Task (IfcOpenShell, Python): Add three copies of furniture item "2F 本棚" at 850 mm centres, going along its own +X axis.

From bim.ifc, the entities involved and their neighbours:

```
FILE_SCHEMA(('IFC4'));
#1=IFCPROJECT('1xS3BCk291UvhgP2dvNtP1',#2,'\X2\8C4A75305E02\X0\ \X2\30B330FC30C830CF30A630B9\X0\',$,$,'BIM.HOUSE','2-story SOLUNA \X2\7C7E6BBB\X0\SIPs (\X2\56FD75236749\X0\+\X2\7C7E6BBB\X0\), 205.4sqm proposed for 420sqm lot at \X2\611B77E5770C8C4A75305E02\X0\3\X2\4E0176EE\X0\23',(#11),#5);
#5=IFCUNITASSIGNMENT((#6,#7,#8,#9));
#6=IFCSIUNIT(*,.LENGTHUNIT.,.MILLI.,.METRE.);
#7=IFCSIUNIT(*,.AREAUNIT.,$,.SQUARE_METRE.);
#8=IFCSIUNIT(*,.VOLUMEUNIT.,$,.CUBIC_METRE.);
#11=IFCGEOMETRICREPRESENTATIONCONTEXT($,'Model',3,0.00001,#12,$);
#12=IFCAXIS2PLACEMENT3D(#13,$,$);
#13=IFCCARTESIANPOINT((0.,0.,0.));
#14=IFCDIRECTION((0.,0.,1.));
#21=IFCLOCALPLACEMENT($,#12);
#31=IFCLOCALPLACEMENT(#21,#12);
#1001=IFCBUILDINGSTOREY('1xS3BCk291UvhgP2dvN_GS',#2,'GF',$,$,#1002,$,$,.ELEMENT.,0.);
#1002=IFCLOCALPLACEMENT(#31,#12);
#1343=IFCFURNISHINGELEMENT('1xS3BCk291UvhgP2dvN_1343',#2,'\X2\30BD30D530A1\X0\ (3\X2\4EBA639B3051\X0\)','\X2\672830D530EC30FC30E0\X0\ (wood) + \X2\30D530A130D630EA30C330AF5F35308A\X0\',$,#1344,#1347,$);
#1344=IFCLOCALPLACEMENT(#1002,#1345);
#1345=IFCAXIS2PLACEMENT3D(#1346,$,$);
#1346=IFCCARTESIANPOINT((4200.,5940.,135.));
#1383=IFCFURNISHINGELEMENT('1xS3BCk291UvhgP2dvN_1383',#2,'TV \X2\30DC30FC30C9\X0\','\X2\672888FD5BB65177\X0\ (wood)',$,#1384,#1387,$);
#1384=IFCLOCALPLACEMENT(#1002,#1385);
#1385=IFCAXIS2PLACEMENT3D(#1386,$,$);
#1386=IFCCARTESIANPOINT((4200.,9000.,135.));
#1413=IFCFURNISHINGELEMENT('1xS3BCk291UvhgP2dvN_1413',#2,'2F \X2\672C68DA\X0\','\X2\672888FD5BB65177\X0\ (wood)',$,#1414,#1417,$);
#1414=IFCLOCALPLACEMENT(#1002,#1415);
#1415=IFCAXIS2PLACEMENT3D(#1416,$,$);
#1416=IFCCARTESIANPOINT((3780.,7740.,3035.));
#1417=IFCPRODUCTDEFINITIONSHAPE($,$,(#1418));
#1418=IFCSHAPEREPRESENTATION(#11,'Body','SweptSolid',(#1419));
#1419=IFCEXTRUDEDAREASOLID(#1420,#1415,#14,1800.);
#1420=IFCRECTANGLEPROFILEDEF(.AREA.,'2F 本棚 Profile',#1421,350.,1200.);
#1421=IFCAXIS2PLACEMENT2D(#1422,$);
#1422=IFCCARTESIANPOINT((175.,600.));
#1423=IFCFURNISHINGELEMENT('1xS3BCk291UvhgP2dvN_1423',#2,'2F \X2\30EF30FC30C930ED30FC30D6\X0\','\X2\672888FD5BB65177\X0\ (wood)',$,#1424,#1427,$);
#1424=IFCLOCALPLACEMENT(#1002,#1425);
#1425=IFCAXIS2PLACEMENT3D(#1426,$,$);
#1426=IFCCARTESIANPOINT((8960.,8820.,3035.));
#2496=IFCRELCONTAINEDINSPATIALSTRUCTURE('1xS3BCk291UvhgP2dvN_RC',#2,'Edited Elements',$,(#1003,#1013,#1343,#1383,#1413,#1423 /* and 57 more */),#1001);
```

```python
import ifcopenshell
import ifcopenshell.api.geometry
import ifcopenshell.api.root
import ifcopenshell.util.element
import ifcopenshell.util.placement
import ifcopenshell.util.unit

model = ifcopenshell.open("bim.ifc")
unit_scale = ifcopenshell.util.unit.calculate_unit_scale(model)


def reuse_history(source, copy):
    """copy_class also copies each property set's owner history, people and application; keep the originals."""
    for rel in copy.IsDefinedBy:
        if rel.is_a("IfcRelDefinesByProperties") and (history := rel.RelatingPropertyDefinition.OwnerHistory):
            rel.RelatingPropertyDefinition.OwnerHistory = source.OwnerHistory
            ifcopenshell.util.element.remove_deep2(model, history)


source = model.by_guid("1xS3BCk291UvhgP2dvN_1413")
base = ifcopenshell.util.placement.get_local_placement(source.ObjectPlacement)
step = base[:3, 0] * 0.85 / unit_scale

for i in range(1, 4):
    copy = ifcopenshell.api.root.copy_class(model, product=source)
    copy.Representation = ifcopenshell.util.element.copy_deep(
        model, source.Representation, exclude=["IfcGeometricRepresentationContext", "IfcRepresentationMap"]
    )
    reuse_history(source, copy)
    matrix = base.copy()
    matrix[:3, 3] += i * step
    print("added at", matrix[:3, 3].round(3) + 0.0)
    ifcopenshell.api.geometry.edit_object_placement(model, product=copy, matrix=matrix, is_si=False)

model.write("bim_v2.ifc")
```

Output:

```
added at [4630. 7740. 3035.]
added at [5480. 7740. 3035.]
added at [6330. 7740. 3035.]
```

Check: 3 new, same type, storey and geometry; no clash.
